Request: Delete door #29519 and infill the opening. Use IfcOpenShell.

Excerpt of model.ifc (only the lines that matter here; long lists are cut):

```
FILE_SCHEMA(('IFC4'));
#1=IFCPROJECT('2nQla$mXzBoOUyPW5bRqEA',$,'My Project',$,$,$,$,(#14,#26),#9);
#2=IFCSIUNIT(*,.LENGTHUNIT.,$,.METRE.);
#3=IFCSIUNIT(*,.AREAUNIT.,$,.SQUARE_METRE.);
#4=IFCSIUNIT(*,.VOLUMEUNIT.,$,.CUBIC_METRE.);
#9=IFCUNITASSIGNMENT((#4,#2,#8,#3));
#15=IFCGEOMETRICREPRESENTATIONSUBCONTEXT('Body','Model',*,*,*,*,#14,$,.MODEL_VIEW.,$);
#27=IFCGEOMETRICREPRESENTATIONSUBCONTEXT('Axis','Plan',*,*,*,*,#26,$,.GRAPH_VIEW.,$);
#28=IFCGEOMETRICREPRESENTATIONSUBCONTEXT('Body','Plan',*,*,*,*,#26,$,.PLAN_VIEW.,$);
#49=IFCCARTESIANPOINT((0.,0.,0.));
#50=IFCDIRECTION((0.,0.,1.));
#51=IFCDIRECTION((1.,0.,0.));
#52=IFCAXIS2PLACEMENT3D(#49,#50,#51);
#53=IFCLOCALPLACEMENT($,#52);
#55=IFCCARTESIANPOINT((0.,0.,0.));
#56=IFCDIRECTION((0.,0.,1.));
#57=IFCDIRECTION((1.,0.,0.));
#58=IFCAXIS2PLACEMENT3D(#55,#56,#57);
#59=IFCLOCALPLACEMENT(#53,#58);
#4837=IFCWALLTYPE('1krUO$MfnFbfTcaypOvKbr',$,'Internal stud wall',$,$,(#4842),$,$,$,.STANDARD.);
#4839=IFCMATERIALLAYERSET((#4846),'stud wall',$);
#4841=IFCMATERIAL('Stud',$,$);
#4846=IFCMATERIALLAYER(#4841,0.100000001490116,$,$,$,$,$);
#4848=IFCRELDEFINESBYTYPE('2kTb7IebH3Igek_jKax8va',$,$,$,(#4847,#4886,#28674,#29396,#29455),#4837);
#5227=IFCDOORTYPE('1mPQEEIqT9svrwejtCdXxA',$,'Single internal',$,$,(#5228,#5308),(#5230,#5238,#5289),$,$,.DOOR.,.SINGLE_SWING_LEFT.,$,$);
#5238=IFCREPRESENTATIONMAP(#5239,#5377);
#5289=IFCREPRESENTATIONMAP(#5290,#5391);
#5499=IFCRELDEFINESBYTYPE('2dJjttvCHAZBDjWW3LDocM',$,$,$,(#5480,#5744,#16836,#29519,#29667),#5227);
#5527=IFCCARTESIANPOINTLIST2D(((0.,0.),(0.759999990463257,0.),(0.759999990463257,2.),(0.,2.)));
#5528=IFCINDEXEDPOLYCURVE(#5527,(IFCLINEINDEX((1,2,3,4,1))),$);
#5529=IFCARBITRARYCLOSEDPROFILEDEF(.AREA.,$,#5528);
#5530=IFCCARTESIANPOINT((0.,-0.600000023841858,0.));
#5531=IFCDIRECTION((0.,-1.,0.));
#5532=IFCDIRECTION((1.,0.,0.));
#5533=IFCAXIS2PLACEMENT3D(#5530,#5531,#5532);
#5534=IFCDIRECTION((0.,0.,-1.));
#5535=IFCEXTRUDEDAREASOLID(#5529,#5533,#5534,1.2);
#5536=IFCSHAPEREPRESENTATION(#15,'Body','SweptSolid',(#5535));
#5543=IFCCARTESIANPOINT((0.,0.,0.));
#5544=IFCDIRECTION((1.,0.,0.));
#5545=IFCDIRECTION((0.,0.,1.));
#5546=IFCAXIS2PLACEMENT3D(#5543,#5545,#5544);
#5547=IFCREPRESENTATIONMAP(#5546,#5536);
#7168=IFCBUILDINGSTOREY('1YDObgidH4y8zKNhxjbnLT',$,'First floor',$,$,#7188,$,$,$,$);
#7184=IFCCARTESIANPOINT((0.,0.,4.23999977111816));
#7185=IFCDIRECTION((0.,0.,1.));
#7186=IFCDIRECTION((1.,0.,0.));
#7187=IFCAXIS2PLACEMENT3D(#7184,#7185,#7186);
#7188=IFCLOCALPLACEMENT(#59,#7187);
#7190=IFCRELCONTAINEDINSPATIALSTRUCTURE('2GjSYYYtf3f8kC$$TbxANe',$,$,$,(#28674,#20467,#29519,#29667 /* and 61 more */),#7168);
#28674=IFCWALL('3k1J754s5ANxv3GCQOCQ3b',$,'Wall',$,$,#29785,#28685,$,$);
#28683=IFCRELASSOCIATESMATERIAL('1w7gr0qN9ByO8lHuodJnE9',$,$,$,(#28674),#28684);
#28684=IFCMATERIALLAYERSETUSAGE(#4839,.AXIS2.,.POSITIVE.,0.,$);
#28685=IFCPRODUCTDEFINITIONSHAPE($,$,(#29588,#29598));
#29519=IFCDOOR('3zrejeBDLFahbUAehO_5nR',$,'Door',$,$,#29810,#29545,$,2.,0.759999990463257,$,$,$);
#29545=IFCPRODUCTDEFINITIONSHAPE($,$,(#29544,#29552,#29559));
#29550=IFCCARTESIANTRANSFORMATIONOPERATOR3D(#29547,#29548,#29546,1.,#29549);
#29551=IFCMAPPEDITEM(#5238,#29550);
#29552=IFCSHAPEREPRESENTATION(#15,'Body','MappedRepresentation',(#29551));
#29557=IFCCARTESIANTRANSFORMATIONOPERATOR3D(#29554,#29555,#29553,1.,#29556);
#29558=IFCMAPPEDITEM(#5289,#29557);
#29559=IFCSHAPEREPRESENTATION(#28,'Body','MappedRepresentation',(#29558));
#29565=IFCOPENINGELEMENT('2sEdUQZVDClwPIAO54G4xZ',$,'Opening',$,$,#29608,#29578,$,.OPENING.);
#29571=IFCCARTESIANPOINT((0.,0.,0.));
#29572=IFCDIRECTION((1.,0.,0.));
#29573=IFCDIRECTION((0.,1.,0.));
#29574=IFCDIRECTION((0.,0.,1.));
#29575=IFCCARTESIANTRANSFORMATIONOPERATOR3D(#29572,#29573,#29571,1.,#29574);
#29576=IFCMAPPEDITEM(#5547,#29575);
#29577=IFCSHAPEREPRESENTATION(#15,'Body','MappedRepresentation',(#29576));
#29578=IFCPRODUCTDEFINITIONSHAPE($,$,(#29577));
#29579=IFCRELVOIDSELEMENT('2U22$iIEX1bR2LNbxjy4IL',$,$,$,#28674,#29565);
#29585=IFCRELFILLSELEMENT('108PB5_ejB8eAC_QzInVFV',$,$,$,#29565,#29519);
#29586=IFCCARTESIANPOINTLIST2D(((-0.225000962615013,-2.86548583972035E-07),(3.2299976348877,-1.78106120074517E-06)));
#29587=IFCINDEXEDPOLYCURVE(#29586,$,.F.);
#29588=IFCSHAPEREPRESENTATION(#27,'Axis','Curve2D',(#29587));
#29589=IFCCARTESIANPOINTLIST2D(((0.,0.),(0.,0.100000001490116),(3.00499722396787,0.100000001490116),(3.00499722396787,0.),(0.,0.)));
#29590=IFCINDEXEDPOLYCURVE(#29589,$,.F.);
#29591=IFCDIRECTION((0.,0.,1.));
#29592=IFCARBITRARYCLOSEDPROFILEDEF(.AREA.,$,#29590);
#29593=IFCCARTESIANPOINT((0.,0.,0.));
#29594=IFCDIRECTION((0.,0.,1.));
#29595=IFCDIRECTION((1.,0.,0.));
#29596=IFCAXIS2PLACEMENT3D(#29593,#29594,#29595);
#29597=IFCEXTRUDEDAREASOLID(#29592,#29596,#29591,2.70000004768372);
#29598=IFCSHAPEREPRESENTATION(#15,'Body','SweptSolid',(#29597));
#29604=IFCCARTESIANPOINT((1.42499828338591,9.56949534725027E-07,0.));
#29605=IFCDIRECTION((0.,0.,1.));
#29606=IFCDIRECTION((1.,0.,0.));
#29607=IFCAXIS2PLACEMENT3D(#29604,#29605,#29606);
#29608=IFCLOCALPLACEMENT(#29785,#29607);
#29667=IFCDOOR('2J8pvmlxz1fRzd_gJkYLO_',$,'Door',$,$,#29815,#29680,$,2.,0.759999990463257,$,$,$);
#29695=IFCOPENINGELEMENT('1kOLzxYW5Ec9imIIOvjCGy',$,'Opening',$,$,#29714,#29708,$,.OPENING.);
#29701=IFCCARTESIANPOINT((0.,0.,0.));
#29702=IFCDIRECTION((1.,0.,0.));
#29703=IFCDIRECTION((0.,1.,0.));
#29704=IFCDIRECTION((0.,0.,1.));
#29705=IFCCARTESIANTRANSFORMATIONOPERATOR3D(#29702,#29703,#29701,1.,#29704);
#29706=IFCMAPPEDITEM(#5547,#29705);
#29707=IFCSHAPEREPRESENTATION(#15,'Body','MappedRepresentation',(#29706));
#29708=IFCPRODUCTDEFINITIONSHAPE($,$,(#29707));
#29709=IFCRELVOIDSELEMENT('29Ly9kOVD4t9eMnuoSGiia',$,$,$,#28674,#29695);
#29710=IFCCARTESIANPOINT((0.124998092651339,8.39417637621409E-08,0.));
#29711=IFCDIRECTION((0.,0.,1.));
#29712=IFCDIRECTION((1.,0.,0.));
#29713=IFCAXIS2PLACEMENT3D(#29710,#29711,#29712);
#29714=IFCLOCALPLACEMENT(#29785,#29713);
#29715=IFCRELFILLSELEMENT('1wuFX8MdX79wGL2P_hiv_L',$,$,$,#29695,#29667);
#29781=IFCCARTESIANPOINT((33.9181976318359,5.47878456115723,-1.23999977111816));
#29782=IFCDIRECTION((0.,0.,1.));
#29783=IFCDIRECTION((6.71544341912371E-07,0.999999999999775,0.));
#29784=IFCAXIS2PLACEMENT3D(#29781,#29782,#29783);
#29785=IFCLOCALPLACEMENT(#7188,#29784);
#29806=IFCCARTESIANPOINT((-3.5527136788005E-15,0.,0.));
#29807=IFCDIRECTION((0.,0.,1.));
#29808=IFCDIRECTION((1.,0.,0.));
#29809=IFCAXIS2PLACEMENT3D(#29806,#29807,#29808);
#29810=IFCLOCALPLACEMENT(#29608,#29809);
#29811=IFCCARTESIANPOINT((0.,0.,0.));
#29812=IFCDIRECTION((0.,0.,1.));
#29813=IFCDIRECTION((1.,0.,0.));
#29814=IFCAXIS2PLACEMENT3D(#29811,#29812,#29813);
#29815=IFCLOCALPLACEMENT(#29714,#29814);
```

```python
import ifcopenshell
import ifcopenshell.api.feature
import ifcopenshell.api.root
import ifcopenshell.geom
import ifcopenshell.util.shape

model = ifcopenshell.open("model.ifc")
settings = ifcopenshell.geom.settings()


def volume(element):
    """Net volume in cubic metres, openings subtracted."""
    shape = ifcopenshell.geom.create_shape(settings, element)
    return ifcopenshell.util.shape.get_volume(shape.geometry)


door = model.by_id(29519)
opening = door.FillsVoids[0].RelatingOpeningElement
wall = opening.VoidsElements[0].RelatingBuildingElement
before = volume(wall)

ifcopenshell.api.root.remove_product(model, product=door)
ifcopenshell.api.feature.remove_feature(model, feature=opening)

after = volume(wall)

print(f"wall volume {before:.3f} -> {after:.3f} m3")

model.write("model_updated.ifc")
```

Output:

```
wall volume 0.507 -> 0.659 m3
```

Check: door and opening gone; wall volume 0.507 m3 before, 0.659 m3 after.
